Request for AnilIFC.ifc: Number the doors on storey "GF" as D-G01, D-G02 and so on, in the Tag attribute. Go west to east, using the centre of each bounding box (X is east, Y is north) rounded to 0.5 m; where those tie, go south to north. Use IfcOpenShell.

First a look at what the model holds.

```python
import ifcopenshell
import ifcopenshell.util.element
import ifcopenshell.util.placement

model = ifcopenshell.open("AnilIFC.ifc")
print(model.schema)
storey = next(s for s in model.by_type("IfcBuildingStorey") if s.Name == "GF")
doors = [e for e in ifcopenshell.util.element.get_decomposition(storey) if e.is_a("IfcDoor")]
for e in sorted(doors, key=lambda e: e.id()):
    origin = ifcopenshell.util.placement.get_local_placement(e.ObjectPlacement)[:3, 3]
    print(e.id(), e.Tag, e.Name, origin.round(2) + 0.0, sep=" | ")
```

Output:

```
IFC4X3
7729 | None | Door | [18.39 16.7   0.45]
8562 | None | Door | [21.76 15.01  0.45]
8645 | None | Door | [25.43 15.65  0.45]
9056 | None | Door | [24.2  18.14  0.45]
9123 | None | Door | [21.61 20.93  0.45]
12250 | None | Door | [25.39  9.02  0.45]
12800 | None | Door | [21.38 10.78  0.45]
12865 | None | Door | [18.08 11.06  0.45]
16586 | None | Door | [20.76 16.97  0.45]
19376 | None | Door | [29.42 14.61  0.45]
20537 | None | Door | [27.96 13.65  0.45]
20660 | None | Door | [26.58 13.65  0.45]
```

```python
import ifcopenshell
import ifcopenshell.geom
import ifcopenshell.util.element
import ifcopenshell.util.shape

model = ifcopenshell.open("AnilIFC.ifc")
settings = ifcopenshell.geom.settings()
settings.set("use-world-coords", True)


def centre(element):
    shape = ifcopenshell.geom.create_shape(settings, element)
    return ifcopenshell.util.shape.get_bbox_centroid(shape.geometry)


storey = next(s for s in model.by_type("IfcBuildingStorey") if s.Name == "GF")
doors = [e for e in ifcopenshell.util.element.get_decomposition(storey) if e.is_a("IfcDoor")]

# Insertion points can sit at a corner or the storey origin, so sort by the geometry (in metres).
centres = {e: centre(e) for e in doors}
doors.sort(key=lambda e: (round(centres[e][0] / 0.5), centres[e][1]))

for i, e in enumerate(doors, start=1):
    number = f"D-G{i:02d}"
    e.Tag = number
    print(e.id(), number)

model.write("AnilIFC-out.ifc")
```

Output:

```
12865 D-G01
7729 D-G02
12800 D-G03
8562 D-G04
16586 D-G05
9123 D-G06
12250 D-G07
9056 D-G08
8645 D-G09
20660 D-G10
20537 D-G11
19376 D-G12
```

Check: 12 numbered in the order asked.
